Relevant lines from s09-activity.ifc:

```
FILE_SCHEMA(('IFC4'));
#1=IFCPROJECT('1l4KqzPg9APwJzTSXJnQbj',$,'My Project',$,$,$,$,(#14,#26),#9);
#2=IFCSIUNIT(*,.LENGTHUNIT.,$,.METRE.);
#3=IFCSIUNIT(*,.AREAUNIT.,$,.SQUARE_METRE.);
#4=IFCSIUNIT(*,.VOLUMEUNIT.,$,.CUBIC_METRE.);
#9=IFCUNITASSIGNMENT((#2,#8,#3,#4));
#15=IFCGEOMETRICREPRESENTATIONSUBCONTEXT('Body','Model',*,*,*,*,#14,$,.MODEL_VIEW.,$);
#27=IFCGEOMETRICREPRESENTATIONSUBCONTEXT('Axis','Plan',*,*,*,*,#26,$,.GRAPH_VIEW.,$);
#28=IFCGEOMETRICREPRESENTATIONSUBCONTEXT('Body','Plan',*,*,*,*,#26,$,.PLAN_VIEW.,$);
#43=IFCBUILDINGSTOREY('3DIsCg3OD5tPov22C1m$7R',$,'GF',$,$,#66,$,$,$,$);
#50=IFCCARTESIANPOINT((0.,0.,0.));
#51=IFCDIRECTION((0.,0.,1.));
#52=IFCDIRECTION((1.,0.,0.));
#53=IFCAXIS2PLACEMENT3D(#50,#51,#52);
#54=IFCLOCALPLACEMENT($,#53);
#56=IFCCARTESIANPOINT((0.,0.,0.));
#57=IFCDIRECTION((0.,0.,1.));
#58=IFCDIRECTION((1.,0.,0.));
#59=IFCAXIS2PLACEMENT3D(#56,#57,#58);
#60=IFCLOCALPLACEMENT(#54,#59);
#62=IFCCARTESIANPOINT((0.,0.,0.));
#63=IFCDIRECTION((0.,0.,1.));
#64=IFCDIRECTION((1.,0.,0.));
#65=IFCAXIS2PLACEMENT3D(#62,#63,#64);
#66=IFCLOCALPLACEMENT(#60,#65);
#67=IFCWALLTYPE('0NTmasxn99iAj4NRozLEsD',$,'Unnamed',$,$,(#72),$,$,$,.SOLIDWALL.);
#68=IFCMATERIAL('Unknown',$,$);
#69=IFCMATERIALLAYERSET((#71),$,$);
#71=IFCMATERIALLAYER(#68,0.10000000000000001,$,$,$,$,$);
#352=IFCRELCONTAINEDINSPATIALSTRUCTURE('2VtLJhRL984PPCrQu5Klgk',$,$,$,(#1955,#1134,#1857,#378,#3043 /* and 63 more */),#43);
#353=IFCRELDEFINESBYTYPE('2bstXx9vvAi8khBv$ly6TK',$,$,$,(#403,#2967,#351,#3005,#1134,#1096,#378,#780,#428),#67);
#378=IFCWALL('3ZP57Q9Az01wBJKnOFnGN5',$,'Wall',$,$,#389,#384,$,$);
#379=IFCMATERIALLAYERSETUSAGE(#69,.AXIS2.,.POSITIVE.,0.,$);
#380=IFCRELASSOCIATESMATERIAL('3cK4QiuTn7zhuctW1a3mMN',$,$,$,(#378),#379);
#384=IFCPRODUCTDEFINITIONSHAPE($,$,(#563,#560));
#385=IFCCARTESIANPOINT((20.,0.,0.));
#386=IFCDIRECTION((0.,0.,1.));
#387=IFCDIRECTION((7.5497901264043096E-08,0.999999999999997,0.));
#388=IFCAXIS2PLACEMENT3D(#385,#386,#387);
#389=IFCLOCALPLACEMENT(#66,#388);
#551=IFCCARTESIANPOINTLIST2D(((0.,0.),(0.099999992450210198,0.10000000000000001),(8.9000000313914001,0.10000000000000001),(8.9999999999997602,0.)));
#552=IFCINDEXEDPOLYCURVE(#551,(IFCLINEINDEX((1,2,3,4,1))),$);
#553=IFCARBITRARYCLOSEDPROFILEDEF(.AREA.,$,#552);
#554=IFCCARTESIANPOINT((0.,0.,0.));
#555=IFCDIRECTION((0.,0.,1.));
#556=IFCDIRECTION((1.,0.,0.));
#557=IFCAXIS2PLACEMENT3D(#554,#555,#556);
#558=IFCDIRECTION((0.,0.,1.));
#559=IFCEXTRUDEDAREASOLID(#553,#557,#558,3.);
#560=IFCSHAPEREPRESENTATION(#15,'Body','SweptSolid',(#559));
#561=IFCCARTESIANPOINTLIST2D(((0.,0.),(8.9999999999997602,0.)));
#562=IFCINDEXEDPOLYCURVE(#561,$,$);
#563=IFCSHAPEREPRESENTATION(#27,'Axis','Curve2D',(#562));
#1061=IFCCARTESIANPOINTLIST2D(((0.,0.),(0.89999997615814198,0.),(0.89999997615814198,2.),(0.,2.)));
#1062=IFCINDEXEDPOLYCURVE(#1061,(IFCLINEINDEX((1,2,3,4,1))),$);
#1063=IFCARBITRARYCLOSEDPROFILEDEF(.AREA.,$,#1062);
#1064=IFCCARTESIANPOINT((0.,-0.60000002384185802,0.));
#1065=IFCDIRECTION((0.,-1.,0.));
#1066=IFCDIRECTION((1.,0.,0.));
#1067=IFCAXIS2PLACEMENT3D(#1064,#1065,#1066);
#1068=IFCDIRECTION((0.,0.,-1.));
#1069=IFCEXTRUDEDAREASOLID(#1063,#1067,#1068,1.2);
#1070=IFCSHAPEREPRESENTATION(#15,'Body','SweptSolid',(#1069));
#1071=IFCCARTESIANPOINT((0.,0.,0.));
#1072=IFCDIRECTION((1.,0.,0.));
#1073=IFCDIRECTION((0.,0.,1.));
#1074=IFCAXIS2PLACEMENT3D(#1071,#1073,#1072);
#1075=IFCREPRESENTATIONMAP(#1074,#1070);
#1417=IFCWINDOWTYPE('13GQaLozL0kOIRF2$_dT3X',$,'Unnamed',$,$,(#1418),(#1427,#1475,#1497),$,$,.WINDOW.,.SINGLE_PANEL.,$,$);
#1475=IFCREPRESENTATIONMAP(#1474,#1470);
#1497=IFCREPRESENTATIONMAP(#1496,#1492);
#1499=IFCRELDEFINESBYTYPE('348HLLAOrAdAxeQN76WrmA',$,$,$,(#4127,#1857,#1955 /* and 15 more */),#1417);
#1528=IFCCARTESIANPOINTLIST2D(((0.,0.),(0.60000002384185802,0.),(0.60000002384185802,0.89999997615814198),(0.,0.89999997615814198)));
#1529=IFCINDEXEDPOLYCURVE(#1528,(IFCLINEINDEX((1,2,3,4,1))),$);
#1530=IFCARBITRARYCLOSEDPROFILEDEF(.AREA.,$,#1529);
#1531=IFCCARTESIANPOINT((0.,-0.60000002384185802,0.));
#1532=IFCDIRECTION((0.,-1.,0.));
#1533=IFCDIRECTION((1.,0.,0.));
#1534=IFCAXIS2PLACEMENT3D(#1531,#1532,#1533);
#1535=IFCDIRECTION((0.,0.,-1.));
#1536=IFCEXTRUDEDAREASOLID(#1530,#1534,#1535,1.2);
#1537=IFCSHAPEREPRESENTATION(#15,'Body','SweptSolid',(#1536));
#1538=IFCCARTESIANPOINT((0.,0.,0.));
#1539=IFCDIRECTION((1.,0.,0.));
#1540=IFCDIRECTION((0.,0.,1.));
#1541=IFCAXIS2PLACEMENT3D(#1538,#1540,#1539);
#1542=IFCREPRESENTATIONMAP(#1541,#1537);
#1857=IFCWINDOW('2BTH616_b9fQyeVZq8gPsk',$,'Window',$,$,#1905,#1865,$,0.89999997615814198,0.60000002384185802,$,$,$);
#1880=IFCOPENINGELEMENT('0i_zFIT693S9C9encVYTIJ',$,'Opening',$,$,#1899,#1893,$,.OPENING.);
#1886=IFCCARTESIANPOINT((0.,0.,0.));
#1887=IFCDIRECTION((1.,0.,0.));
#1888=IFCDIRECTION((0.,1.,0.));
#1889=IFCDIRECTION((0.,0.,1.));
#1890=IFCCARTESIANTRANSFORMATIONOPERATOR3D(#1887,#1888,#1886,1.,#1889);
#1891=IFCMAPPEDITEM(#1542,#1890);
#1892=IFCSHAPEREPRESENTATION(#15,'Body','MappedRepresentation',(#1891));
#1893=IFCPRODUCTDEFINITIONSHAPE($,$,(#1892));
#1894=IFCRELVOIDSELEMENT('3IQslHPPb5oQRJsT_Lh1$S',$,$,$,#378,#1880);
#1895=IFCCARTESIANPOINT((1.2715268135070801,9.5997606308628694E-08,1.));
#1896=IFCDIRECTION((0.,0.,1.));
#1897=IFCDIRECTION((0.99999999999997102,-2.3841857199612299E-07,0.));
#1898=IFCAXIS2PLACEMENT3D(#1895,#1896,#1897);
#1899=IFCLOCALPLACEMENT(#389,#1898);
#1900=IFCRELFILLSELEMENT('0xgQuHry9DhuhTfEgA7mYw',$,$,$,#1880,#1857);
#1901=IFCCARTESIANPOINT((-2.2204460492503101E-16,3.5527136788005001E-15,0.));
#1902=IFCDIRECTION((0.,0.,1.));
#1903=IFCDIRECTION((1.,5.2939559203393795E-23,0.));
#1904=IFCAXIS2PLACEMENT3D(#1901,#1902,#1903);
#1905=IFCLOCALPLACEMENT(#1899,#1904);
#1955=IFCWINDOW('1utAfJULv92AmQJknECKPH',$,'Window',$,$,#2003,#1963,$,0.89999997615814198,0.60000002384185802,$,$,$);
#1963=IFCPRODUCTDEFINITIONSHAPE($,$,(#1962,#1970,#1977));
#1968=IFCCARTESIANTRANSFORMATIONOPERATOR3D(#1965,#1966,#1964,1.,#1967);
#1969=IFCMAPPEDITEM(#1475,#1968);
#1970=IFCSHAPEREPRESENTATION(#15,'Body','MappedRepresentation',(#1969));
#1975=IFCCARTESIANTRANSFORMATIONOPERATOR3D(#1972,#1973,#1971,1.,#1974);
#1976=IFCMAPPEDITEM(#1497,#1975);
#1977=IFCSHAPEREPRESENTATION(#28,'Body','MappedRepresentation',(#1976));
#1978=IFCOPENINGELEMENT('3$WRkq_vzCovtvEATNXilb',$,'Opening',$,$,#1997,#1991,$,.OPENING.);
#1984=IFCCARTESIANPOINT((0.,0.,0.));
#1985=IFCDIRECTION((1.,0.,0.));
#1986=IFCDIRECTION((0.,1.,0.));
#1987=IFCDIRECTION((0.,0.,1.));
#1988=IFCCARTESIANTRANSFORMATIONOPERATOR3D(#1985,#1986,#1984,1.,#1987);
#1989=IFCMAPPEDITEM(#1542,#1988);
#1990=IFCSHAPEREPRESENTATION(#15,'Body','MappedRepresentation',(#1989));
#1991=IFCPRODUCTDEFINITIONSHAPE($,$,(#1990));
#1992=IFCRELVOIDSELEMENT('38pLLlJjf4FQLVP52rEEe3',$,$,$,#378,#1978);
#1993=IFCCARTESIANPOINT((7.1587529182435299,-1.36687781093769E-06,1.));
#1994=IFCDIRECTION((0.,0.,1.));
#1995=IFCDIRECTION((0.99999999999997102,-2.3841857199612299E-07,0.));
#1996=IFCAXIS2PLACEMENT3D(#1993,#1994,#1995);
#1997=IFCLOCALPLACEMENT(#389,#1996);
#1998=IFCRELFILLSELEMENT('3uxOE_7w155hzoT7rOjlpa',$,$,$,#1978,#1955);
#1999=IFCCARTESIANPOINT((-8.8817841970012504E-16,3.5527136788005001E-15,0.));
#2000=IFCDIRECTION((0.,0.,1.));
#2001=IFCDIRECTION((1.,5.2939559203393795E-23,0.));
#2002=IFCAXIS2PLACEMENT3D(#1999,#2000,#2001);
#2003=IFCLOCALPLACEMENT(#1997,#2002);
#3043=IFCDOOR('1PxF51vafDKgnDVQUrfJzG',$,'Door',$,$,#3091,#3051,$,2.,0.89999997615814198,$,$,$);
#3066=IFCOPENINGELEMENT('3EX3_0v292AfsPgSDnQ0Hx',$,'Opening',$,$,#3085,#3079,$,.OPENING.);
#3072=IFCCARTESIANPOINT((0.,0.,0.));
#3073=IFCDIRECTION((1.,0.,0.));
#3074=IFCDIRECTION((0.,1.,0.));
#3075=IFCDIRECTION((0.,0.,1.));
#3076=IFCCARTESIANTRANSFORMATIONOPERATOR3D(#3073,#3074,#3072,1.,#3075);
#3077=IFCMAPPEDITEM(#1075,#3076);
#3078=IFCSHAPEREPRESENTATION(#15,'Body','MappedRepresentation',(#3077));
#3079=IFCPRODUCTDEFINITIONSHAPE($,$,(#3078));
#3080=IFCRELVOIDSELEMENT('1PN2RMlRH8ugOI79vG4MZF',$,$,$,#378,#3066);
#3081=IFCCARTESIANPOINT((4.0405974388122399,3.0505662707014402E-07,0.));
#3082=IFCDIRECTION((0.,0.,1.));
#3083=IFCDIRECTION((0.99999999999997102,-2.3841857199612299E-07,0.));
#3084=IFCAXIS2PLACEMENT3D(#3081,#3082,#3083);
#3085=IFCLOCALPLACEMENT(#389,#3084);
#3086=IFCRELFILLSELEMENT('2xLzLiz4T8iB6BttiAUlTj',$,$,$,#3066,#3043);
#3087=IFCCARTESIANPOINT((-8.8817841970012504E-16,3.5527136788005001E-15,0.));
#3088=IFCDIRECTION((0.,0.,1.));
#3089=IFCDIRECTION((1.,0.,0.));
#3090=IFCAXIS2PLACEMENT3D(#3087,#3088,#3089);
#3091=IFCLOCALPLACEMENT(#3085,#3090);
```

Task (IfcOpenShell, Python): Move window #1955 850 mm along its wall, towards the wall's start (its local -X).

```python
import ifcopenshell
import ifcopenshell.api.geometry
import ifcopenshell.util.placement

model = ifcopenshell.open("s09-activity.ifc")

window = model.by_guid("1utAfJULv92AmQJknECKPH")
opening = window.FillsVoids[0].RelatingOpeningElement
wall = opening.VoidsElements[0].RelatingBuildingElement

wall_matrix = ifcopenshell.util.placement.get_local_placement(wall.ObjectPlacement)
shift = wall_matrix[:3, 0] * -0.85
before = ifcopenshell.util.placement.get_local_placement(window.ObjectPlacement)[:3, 3].copy()

# The window is placed relative to its opening, so it follows when the opening moves.
matrix = ifcopenshell.util.placement.get_local_placement(opening.ObjectPlacement)
matrix[:3, 3] += shift
ifcopenshell.api.geometry.edit_object_placement(
    model, product=opening, matrix=matrix, is_si=False, should_transform_children=True
)

after = ifcopenshell.util.placement.get_local_placement(window.ObjectPlacement)[:3, 3]
print("window moved by", (after - before).round(3) + 0.0)

model.write("s09-activity_v2.ifc")
```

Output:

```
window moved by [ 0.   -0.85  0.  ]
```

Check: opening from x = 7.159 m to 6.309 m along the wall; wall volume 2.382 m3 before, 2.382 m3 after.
